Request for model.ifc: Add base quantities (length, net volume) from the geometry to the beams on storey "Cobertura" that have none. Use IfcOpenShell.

First a look at what the model holds.

```python
import ifcopenshell
import ifcopenshell.util.element
import ifcopenshell.util.unit

model = ifcopenshell.open("model.ifc")
print(model.schema)
for unit_type in ("LENGTHUNIT", "AREAUNIT", "VOLUMEUNIT"):
    print(unit_type, ifcopenshell.util.unit.calculate_unit_scale(model, unit_type))
storey = next(s for s in model.by_type("IfcBuildingStorey") if s.Name == "Cobertura")
beams = [e for e in ifcopenshell.util.element.get_decomposition(storey) if e.is_a("IfcBeam")]
for e in sorted(beams, key=lambda e: e.id()):
    print(e.id(), e.is_a(), e.Name, list(ifcopenshell.util.element.get_psets(e, qtos_only=True)), sep=" | ")
```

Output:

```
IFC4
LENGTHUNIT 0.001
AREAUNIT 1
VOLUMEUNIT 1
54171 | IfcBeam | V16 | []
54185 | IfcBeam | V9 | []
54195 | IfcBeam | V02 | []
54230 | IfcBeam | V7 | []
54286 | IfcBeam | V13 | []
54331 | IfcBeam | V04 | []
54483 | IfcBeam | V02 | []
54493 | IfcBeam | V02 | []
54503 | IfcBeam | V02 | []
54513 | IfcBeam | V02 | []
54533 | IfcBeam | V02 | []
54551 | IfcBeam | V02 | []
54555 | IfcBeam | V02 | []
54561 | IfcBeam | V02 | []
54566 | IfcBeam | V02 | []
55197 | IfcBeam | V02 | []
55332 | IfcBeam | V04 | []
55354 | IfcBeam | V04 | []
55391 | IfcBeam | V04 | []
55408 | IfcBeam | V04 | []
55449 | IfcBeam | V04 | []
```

```python
import ifcopenshell
import ifcopenshell.api.pset
import ifcopenshell.geom
import ifcopenshell.util.element
import ifcopenshell.util.shape
import ifcopenshell.util.unit

model = ifcopenshell.open("model.ifc")
unit_scale = ifcopenshell.util.unit.calculate_unit_scale(model)
volume_scale = ifcopenshell.util.unit.calculate_unit_scale(model, "VOLUMEUNIT")
settings = ifcopenshell.geom.settings()

storey = next(s for s in model.by_type("IfcBuildingStorey") if s.Name == "Cobertura")
beams = [e for e in ifcopenshell.util.element.get_decomposition(storey) if e.is_a("IfcBeam")]

for e in sorted(beams, key=lambda e: e.id()):
    if ifcopenshell.util.element.get_psets(e, qtos_only=True, should_inherit=False):
        continue
    # Geometry comes back in metres, in the element's own axes.
    shape = ifcopenshell.geom.create_shape(settings, e)
    values = {
        "Length": ifcopenshell.util.shape.get_max_xyz(shape.geometry) / unit_scale,
        "NetVolume": ifcopenshell.util.shape.get_volume(shape.geometry) / volume_scale,
    }
    qto = ifcopenshell.api.pset.add_qto(model, product=e, name="Qto_BeamBaseQuantities")
    ifcopenshell.api.pset.edit_qto(model, qto=qto, properties=values)
    print(e.id(), {k: round(v, 3) for k, v in values.items()})

model.write("model_updated.ifc")
```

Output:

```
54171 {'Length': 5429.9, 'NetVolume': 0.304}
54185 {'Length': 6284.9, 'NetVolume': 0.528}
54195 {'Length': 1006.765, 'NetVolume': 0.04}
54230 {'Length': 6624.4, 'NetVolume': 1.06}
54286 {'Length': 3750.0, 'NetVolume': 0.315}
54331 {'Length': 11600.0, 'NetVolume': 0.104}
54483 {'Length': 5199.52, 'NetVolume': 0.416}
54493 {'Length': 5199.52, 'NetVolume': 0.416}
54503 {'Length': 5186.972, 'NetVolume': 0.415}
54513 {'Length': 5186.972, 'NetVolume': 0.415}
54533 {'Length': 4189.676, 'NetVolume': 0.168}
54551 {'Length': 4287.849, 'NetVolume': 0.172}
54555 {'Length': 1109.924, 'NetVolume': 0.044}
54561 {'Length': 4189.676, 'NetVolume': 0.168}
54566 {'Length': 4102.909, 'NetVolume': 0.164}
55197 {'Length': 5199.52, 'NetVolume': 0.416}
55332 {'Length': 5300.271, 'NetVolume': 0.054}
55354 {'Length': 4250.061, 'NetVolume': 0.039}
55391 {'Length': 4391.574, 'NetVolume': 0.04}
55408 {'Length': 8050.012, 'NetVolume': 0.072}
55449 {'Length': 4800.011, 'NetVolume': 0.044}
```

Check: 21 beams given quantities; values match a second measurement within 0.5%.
